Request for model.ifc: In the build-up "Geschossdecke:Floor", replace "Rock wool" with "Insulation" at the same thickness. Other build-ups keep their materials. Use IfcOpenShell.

First a look at what the model holds.

```python
import ifcopenshell
import ifcopenshell.util.element

model = ifcopenshell.open("model.ifc")
print(model.schema)
for layer_set in model.by_type("IfcMaterialLayerSet"):
    if layer_set.LayerSetName == "Geschossdecke:Floor":
        for layer in layer_set.MaterialLayers:
            print(layer.id(), layer.Material and layer.Material.Name, layer.LayerThickness, sep=" | ")
        print(len(ifcopenshell.util.element.get_elements_by_material(model, layer_set)), "elements and types use it")
print(sorted(m.Name for m in model.by_type("IfcMaterial") if m.Name)[:60])
```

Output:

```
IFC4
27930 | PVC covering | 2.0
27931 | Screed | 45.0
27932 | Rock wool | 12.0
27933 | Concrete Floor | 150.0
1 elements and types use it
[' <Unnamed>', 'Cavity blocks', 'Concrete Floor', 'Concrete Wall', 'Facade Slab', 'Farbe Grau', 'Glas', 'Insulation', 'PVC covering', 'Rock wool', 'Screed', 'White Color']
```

```python
import ifcopenshell
import ifcopenshell.api.material

model = ifcopenshell.open("model.ifc")

layer_set = next(s for s in model.by_type("IfcMaterialLayerSet") if s.LayerSetName == "Geschossdecke:Floor")
layer = next(l for l in layer_set.MaterialLayers if l.Material and l.Material.Name == "Rock wool")
material = next(m for m in model.by_type("IfcMaterial") if m.Name == "Insulation")

# Point this one layer at the other material; renaming the old one would change it everywhere.
ifcopenshell.api.material.edit_layer(model, layer=layer, attributes={}, material=material)

print([l.Material.Name if l.Material else None for l in layer_set.MaterialLayers])

model.write("model-out.ifc")
```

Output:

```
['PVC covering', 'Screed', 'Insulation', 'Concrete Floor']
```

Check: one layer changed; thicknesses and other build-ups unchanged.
